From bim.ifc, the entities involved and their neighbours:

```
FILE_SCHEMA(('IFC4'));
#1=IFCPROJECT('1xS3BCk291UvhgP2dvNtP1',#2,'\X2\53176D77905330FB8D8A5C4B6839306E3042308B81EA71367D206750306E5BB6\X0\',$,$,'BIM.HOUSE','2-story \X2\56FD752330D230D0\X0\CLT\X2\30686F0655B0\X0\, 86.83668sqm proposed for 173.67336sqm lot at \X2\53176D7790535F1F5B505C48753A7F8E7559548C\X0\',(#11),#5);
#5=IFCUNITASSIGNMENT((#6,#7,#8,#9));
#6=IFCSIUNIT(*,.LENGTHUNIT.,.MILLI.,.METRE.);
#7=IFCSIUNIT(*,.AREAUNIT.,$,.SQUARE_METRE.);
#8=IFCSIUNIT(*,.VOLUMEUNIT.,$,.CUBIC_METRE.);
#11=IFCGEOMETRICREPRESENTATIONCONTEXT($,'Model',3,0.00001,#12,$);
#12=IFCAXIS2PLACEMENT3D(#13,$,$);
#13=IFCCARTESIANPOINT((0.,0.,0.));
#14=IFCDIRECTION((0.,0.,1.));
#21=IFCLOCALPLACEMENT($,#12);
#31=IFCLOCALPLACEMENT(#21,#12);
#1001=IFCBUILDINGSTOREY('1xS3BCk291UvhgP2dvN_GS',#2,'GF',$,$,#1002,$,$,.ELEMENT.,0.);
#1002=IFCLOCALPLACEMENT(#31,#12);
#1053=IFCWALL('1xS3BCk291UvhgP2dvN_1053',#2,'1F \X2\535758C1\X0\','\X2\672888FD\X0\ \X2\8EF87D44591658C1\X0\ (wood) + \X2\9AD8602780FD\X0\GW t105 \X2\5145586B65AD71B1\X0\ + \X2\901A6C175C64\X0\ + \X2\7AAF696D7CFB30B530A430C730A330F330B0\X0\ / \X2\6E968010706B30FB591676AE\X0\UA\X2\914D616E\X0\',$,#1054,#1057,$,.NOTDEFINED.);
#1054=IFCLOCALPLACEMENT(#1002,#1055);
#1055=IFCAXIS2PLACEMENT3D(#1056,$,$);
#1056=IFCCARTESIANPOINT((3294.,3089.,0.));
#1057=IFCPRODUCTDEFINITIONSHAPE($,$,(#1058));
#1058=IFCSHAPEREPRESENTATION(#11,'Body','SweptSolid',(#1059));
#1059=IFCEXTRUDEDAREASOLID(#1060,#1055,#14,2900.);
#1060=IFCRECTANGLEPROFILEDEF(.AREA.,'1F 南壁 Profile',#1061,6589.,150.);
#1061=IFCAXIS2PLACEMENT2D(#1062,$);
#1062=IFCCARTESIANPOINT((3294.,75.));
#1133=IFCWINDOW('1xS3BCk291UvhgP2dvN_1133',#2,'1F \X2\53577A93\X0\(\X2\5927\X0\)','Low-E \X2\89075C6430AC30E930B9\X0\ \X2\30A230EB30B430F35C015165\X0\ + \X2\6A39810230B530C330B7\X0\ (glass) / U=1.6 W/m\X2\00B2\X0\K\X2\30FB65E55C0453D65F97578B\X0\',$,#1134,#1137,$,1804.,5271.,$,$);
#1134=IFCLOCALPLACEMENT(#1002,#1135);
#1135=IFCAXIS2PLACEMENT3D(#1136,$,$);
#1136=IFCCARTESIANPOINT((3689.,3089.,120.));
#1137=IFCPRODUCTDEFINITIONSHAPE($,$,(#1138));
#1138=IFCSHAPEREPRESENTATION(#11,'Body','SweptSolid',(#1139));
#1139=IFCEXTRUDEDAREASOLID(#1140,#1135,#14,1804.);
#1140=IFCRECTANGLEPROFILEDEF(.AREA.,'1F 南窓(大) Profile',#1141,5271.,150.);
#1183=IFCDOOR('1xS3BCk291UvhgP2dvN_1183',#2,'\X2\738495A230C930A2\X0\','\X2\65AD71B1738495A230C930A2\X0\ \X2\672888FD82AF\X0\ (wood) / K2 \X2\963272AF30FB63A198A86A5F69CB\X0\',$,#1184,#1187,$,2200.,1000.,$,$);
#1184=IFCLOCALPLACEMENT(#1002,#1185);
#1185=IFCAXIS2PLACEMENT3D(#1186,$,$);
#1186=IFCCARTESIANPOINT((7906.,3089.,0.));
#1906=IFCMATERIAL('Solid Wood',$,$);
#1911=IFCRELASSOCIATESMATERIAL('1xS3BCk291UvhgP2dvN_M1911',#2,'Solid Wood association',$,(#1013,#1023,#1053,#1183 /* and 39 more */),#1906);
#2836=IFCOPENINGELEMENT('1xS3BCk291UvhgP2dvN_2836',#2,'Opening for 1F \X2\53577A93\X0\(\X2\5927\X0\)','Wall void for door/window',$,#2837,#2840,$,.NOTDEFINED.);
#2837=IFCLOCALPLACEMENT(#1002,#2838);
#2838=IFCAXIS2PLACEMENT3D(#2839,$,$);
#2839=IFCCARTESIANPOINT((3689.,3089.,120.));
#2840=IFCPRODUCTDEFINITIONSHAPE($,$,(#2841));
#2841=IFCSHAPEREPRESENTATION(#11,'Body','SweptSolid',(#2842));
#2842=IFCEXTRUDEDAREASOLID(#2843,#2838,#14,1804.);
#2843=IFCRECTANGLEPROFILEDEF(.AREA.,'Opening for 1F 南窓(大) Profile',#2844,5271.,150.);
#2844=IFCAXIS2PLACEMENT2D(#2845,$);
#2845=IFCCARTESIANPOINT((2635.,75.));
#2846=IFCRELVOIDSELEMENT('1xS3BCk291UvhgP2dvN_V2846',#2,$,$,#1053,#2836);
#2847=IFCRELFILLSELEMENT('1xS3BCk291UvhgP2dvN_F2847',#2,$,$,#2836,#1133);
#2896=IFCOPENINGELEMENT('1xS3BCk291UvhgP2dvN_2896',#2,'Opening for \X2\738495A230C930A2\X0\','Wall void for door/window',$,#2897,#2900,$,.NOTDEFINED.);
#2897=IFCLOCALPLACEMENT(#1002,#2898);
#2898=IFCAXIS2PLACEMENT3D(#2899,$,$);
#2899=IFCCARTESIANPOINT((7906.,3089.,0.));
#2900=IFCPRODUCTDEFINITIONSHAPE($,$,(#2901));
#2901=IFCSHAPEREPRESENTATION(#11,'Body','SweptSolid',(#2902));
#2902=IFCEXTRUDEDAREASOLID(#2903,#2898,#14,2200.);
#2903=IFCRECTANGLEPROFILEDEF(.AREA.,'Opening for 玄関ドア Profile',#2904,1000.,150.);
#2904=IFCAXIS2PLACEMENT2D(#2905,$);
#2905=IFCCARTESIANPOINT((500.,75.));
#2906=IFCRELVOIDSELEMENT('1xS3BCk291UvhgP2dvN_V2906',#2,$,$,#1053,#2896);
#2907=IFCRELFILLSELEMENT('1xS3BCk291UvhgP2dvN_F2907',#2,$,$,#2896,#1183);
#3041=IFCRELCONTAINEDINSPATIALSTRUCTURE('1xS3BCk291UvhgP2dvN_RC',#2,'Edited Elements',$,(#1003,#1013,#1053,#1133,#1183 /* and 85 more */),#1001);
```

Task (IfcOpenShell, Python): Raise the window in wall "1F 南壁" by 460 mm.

```python
import numpy as np
import ifcopenshell
import ifcopenshell.api.geometry
import ifcopenshell.util.placement
import ifcopenshell.util.unit

model = ifcopenshell.open("bim.ifc")
unit_scale = ifcopenshell.util.unit.calculate_unit_scale(model)

window = model.by_guid("1xS3BCk291UvhgP2dvN_1133")
opening = window.FillsVoids[0].RelatingOpeningElement
dz = 460.0

shift = np.array([0.0, 0.0, dz])
# The window is not placed relative to its opening, so move both.
for product in (opening, window):
    matrix = ifcopenshell.util.placement.get_local_placement(product.ObjectPlacement)
    matrix[:3, 3] += shift
    ifcopenshell.api.geometry.edit_object_placement(model, product=product, matrix=matrix, is_si=False)

print(f"moved by {dz * unit_scale:+.3f} m")

model.write("bim_edited.ifc")
```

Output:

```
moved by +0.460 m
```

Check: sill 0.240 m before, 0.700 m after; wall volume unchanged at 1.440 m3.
